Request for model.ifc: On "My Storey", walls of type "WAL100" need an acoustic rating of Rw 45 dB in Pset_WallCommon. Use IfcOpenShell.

First a look at what the model holds.

```python
import ifcopenshell
import ifcopenshell.util.element

model = ifcopenshell.open("model.ifc")
print(model.schema)
storey = next(s for s in model.by_type("IfcBuildingStorey") if s.Name == "My Storey")
walls = [e for e in ifcopenshell.util.element.get_decomposition(storey) if e.is_a("IfcWall")]
seen = {}
for e in walls:
    element_type = ifcopenshell.util.element.get_type(e)
    key = (element_type.Name if element_type != e and element_type else None, ifcopenshell.util.element.get_pset(e, "Pset_WallCommon", "AcousticRating"))
    seen[key] = seen.get(key, 0) + 1
for (name, value), count in sorted(seen.items(), key=str):
    print(count, "x", name, "|", value)
```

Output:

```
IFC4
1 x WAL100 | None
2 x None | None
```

```python
import ifcopenshell
import ifcopenshell.api.pset
import ifcopenshell.util.element

model = ifcopenshell.open("model.ifc")

storey = next(s for s in model.by_type("IfcBuildingStorey") if s.Name == "My Storey")
walls = [e for e in ifcopenshell.util.element.get_decomposition(storey) if e.is_a("IfcWall")]

count = 0
for e in walls:
    element_type = ifcopenshell.util.element.get_type(e)
    if element_type in (None, e) or element_type.Name != "WAL100":
        continue
    # add_pset returns the element's existing set when there is one.
    pset = ifcopenshell.api.pset.add_pset(model, product=e, name="Pset_WallCommon")
    ifcopenshell.api.pset.edit_pset(model, pset=pset, properties={"AcousticRating": "Rw 45 dB"})
    count += 1

print(count, "walls updated")

model.write("model_rev.ifc")
```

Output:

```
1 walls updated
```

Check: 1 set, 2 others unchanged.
